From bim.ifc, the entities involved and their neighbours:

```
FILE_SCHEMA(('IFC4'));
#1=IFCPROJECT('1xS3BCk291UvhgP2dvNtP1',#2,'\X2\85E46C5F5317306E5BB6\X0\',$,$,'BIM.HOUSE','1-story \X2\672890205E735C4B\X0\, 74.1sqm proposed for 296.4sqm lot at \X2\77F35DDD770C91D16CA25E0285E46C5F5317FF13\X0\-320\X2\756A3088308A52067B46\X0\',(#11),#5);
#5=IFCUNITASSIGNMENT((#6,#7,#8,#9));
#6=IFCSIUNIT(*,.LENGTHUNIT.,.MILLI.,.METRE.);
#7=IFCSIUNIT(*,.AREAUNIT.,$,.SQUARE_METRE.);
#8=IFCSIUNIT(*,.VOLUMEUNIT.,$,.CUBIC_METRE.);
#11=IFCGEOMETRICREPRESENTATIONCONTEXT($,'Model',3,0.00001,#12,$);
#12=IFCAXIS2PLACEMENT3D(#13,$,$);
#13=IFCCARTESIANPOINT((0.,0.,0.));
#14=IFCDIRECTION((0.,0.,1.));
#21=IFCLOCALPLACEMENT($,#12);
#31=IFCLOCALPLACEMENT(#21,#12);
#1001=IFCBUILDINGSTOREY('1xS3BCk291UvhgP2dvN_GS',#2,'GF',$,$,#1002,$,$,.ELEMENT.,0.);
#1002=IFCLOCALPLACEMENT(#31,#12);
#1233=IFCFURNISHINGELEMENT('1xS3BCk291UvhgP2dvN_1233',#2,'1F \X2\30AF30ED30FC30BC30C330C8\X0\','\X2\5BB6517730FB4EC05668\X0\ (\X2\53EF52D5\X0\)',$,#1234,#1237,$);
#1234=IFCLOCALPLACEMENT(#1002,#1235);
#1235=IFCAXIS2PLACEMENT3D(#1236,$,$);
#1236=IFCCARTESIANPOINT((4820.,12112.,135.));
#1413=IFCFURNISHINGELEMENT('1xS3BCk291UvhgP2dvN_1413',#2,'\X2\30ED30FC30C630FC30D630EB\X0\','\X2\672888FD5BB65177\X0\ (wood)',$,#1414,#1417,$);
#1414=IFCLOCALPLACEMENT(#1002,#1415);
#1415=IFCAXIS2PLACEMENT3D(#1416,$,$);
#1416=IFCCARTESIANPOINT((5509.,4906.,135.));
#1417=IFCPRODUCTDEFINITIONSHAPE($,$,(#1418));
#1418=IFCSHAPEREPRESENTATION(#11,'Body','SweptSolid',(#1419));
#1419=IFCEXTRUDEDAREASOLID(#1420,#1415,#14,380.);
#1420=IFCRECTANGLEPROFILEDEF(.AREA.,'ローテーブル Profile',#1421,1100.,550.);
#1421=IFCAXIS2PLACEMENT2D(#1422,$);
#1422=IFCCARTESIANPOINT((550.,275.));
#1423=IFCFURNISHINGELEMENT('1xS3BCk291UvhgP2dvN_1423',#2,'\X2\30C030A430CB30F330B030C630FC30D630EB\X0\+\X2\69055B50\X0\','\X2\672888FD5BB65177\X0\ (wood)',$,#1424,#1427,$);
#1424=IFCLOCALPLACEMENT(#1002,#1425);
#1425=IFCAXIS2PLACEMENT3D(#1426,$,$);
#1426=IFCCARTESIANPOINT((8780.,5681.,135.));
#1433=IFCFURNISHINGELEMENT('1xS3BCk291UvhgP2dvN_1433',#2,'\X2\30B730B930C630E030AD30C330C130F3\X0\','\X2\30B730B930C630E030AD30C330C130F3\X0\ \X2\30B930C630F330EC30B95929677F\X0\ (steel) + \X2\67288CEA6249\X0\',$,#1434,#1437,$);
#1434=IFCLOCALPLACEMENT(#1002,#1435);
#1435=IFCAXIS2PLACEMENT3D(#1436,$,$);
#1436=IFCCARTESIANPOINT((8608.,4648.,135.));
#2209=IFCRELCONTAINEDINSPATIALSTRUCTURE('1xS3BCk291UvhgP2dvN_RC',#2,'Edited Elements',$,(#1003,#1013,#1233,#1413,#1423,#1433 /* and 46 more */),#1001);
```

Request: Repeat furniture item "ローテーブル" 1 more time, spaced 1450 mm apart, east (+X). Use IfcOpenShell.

```python
import numpy as np
import ifcopenshell
import ifcopenshell.api.geometry
import ifcopenshell.api.root
import ifcopenshell.util.element
import ifcopenshell.util.placement

model = ifcopenshell.open("bim.ifc")


def reuse_history(source, copy):
    """copy_class also copies each property set's owner history, people and application; keep the originals."""
    for rel in copy.IsDefinedBy:
        if rel.is_a("IfcRelDefinesByProperties") and (history := rel.RelatingPropertyDefinition.OwnerHistory):
            rel.RelatingPropertyDefinition.OwnerHistory = source.OwnerHistory
            ifcopenshell.util.element.remove_deep2(model, history)


source = model.by_guid("1xS3BCk291UvhgP2dvN_1413")
base = ifcopenshell.util.placement.get_local_placement(source.ObjectPlacement)
step = np.array([1.0, 0.0, 0.0]) * 1450.0

for i in range(1, 2):
    copy = ifcopenshell.api.root.copy_class(model, product=source)
    copy.Representation = ifcopenshell.util.element.copy_deep(
        model, source.Representation, exclude=["IfcGeometricRepresentationContext", "IfcRepresentationMap"]
    )
    reuse_history(source, copy)
    matrix = base.copy()
    matrix[:3, 3] += i * step
    print("added at", matrix[:3, 3].round(3) + 0.0)
    ifcopenshell.api.geometry.edit_object_placement(model, product=copy, matrix=matrix, is_si=False)

model.write("bim_v2.ifc")
```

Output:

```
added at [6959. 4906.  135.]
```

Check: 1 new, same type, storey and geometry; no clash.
